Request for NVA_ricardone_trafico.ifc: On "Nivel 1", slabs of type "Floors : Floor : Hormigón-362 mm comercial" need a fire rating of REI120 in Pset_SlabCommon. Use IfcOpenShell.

First a look at what the model holds.

```python
import ifcopenshell
import ifcopenshell.util.element

model = ifcopenshell.open("NVA_ricardone_trafico.ifc")
print(model.schema)
storey = next(s for s in model.by_type("IfcBuildingStorey") if s.Name == "Nivel 1")
slabs = [e for e in ifcopenshell.util.element.get_decomposition(storey) if e.is_a("IfcSlab")]
seen = {}
for e in slabs:
    element_type = ifcopenshell.util.element.get_type(e)
    key = (element_type.Name if element_type != e and element_type else None, ifcopenshell.util.element.get_pset(e, "Pset_SlabCommon", "FireRating"))
    seen[key] = seen.get(key, 0) + 1
for (name, value), count in sorted(seen.items(), key=str):
    print(count, "x", name, "|", value)
```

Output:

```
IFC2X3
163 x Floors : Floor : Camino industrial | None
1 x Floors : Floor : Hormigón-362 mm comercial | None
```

```python
import ifcopenshell
import ifcopenshell.api.pset
import ifcopenshell.util.element

model = ifcopenshell.open("NVA_ricardone_trafico.ifc")

storey = next(s for s in model.by_type("IfcBuildingStorey") if s.Name == "Nivel 1")
slabs = [e for e in ifcopenshell.util.element.get_decomposition(storey) if e.is_a("IfcSlab")]

count = 0
for e in slabs:
    element_type = ifcopenshell.util.element.get_type(e)
    if element_type in (None, e) or element_type.Name != "Floors : Floor : Hormigón-362 mm comercial":
        continue
    # add_pset returns the element's existing set when there is one.
    pset = ifcopenshell.api.pset.add_pset(model, product=e, name="Pset_SlabCommon")
    ifcopenshell.api.pset.edit_pset(model, pset=pset, properties={"FireRating": "REI120"})
    count += 1

print(count, "slabs updated")

model.write("NVA_ricardone_trafico_updated.ifc")
```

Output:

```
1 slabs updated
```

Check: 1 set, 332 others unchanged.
